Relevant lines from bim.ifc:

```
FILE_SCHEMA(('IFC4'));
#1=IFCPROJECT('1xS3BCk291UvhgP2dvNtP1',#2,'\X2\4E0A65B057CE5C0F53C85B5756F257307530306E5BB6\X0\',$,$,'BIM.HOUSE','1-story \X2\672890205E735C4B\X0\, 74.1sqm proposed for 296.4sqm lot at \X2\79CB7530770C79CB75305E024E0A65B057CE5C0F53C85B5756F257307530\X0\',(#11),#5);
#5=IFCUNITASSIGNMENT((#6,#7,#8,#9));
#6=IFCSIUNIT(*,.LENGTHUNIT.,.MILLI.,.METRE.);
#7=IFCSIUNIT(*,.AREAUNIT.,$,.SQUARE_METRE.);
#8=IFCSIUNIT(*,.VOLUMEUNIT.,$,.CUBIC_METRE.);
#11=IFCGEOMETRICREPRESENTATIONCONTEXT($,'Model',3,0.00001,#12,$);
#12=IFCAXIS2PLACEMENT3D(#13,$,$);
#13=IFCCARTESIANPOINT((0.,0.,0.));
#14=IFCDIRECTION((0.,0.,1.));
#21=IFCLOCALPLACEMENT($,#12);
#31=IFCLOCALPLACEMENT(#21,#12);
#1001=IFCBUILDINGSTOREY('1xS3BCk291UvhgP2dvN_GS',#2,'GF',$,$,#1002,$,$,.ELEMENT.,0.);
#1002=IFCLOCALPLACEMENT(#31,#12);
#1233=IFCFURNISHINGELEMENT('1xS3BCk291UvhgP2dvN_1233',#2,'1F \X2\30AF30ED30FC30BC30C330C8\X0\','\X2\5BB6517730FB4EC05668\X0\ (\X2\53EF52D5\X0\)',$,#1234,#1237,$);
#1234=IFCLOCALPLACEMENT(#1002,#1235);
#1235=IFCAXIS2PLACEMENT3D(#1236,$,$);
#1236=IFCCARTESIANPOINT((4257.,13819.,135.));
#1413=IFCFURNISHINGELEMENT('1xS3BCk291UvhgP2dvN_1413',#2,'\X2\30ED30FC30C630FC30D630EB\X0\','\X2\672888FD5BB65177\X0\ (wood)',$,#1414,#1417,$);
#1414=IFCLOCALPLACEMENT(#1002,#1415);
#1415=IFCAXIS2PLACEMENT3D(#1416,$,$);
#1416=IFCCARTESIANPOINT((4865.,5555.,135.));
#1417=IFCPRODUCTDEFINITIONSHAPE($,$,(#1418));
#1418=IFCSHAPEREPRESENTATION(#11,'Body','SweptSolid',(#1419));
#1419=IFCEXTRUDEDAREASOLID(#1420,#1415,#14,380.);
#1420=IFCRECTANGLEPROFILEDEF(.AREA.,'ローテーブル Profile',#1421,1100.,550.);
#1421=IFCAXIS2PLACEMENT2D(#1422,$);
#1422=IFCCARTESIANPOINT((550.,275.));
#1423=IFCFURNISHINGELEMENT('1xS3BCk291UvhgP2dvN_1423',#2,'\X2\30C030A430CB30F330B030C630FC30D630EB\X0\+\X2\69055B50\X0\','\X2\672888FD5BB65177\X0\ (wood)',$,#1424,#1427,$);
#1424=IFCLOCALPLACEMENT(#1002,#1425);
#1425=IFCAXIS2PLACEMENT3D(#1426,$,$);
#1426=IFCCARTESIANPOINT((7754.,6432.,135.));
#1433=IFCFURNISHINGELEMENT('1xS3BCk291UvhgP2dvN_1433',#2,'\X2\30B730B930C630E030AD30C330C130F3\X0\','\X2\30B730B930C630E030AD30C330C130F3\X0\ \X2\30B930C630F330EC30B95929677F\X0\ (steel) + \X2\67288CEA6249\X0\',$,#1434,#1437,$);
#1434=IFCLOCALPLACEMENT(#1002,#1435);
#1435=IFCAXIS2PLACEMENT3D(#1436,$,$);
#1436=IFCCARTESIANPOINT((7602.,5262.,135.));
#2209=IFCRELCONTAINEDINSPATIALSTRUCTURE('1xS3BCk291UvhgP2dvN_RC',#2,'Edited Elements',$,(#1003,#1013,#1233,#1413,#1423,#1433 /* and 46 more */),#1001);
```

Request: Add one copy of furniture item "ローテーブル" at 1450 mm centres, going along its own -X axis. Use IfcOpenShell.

```python
import ifcopenshell
import ifcopenshell.api.geometry
import ifcopenshell.api.root
import ifcopenshell.util.element
import ifcopenshell.util.placement

model = ifcopenshell.open("bim.ifc")


def reuse_history(source, copy):
    """copy_class also copies each property set's owner history, people and application; keep the originals."""
    for rel in copy.IsDefinedBy:
        if rel.is_a("IfcRelDefinesByProperties") and (history := rel.RelatingPropertyDefinition.OwnerHistory):
            rel.RelatingPropertyDefinition.OwnerHistory = source.OwnerHistory
            ifcopenshell.util.element.remove_deep2(model, history)


source = model.by_id(1413)
base = ifcopenshell.util.placement.get_local_placement(source.ObjectPlacement)
step = -base[:3, 0] * 1450.0

for i in range(1, 2):
    copy = ifcopenshell.api.root.copy_class(model, product=source)
    copy.Representation = ifcopenshell.util.element.copy_deep(
        model, source.Representation, exclude=["IfcGeometricRepresentationContext", "IfcRepresentationMap"]
    )
    reuse_history(source, copy)
    matrix = base.copy()
    matrix[:3, 3] += i * step
    print("added at", matrix[:3, 3].round(3) + 0.0)
    ifcopenshell.api.geometry.edit_object_placement(model, product=copy, matrix=matrix, is_si=False)

model.write("bim_updated.ifc")
```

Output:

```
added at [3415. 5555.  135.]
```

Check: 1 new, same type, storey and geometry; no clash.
